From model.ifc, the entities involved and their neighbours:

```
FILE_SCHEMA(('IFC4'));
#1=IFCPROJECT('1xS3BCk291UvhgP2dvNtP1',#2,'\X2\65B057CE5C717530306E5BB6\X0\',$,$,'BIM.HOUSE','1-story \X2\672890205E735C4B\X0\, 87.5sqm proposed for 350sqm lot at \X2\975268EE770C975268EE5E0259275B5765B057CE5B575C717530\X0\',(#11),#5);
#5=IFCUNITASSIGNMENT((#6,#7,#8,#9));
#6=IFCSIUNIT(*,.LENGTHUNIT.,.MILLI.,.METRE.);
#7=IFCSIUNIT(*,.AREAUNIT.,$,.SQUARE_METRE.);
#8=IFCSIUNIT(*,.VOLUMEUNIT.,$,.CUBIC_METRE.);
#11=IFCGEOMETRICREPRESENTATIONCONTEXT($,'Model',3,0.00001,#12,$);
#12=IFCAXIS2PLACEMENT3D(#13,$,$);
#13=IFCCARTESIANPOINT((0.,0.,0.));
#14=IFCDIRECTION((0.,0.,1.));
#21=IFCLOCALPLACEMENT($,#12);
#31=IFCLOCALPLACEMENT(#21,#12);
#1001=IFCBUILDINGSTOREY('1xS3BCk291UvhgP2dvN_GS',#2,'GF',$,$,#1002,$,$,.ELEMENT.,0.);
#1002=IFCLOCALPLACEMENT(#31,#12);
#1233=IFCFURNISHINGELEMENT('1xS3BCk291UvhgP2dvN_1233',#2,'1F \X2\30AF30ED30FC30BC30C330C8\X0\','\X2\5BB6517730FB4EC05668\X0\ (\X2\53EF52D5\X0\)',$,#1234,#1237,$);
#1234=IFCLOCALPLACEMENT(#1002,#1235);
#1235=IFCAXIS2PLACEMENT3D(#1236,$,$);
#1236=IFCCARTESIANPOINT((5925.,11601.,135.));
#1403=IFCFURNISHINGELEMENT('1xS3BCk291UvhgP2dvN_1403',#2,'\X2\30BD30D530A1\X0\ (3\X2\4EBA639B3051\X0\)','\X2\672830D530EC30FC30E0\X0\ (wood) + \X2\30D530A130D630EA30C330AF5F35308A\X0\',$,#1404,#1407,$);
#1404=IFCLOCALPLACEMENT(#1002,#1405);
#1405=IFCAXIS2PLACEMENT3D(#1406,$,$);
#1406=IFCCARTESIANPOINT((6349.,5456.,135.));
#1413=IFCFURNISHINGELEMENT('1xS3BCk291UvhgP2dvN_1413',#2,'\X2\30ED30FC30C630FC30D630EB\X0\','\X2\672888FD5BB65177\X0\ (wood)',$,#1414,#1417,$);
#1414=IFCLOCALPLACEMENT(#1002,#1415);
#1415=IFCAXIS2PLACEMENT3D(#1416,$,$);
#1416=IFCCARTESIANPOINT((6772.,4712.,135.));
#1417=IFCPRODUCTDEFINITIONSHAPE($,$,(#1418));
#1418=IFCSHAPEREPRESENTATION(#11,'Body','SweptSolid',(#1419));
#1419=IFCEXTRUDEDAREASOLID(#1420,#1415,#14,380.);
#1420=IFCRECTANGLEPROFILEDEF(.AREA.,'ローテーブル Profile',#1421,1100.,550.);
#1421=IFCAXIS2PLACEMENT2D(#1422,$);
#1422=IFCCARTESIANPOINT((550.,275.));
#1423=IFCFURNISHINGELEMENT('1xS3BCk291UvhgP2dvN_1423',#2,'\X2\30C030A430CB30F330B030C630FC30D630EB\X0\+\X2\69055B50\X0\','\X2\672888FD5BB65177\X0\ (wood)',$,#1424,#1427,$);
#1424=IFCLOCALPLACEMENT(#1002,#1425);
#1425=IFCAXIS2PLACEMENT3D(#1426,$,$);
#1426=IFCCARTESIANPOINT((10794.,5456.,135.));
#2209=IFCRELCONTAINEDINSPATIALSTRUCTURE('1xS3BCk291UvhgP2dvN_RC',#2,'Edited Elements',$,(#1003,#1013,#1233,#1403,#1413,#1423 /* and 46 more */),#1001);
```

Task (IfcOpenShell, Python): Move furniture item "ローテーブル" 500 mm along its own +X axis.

```python
import ifcopenshell
import ifcopenshell.api.geometry
import ifcopenshell.util.placement
import ifcopenshell.util.unit

model = ifcopenshell.open("model.ifc")
unit_scale = ifcopenshell.util.unit.calculate_unit_scale(model)

item = model.by_guid("1xS3BCk291UvhgP2dvN_1413")
matrix = ifcopenshell.util.placement.get_local_placement(item.ObjectPlacement)
matrix[:3, 3] += matrix[:3, 0] * 0.5 / unit_scale
ifcopenshell.api.geometry.edit_object_placement(model, product=item, matrix=matrix, is_si=False)

print(ifcopenshell.util.placement.get_local_placement(item.ObjectPlacement).round(3) + 0.0)

model.write("model_v2.ifc")
```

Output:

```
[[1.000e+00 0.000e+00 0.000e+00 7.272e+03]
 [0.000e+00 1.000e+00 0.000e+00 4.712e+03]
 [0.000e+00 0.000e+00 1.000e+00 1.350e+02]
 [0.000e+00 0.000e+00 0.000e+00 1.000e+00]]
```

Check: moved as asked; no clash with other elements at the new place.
